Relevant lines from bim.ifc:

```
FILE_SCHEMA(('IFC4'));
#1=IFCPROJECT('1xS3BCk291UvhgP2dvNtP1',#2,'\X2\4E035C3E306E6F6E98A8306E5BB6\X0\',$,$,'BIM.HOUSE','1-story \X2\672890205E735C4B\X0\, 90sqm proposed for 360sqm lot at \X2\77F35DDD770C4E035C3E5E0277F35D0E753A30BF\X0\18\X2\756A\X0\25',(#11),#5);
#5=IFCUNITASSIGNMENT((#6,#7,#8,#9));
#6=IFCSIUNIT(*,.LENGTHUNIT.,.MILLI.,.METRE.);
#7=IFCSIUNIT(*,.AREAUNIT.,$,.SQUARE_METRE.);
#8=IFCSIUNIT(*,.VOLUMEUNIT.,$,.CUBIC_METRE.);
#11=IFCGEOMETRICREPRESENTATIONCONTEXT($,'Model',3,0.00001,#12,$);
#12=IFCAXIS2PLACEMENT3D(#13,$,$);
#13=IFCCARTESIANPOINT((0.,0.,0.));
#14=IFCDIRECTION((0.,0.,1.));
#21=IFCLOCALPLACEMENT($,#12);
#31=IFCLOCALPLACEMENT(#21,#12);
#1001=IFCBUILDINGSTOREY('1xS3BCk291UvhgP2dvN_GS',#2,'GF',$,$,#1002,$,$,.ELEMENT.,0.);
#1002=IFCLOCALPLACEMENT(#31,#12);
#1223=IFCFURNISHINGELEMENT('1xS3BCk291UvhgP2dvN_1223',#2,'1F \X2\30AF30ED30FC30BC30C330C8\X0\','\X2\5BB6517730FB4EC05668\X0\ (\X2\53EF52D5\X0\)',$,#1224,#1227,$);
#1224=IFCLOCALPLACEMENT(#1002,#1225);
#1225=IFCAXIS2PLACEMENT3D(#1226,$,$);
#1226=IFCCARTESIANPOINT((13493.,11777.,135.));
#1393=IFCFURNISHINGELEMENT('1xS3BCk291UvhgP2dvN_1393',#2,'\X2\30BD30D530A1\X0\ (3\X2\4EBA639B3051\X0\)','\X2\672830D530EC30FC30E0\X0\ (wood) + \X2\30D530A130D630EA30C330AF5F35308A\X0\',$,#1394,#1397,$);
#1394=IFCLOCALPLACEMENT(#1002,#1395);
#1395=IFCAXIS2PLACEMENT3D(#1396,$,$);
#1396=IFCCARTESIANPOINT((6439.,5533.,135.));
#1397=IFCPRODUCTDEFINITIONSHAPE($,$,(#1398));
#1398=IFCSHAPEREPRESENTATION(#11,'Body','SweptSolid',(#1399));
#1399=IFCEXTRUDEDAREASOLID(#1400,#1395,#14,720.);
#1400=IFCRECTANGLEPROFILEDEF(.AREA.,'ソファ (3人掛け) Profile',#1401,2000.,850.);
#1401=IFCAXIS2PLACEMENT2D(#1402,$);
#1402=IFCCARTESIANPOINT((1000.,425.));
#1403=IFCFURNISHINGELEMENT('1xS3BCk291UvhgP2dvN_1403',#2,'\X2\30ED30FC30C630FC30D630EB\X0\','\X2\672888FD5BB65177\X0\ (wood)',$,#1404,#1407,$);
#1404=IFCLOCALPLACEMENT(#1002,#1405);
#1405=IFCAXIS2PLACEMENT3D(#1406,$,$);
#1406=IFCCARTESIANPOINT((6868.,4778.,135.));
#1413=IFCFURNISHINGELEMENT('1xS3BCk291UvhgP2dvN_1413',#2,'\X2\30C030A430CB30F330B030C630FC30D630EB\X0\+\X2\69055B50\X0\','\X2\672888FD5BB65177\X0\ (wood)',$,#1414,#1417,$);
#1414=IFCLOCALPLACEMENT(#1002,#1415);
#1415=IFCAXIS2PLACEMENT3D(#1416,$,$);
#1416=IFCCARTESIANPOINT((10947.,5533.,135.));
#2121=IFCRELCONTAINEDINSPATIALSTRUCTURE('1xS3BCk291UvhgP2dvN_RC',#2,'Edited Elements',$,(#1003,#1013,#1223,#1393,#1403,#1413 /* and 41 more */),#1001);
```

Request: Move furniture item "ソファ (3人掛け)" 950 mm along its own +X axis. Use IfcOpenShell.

```python
import ifcopenshell
import ifcopenshell.api.geometry
import ifcopenshell.util.placement

model = ifcopenshell.open("bim.ifc")

item = model.by_guid("1xS3BCk291UvhgP2dvN_1393")
matrix = ifcopenshell.util.placement.get_local_placement(item.ObjectPlacement)
matrix[:3, 3] += matrix[:3, 0] * 950.0
ifcopenshell.api.geometry.edit_object_placement(model, product=item, matrix=matrix, is_si=False)

print(ifcopenshell.util.placement.get_local_placement(item.ObjectPlacement).round(3) + 0.0)

model.write("bim_edited.ifc")
```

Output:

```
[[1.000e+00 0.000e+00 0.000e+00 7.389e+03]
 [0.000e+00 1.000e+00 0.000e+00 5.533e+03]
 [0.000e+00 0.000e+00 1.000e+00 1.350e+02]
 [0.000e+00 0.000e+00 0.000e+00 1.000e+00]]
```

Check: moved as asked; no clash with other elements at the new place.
